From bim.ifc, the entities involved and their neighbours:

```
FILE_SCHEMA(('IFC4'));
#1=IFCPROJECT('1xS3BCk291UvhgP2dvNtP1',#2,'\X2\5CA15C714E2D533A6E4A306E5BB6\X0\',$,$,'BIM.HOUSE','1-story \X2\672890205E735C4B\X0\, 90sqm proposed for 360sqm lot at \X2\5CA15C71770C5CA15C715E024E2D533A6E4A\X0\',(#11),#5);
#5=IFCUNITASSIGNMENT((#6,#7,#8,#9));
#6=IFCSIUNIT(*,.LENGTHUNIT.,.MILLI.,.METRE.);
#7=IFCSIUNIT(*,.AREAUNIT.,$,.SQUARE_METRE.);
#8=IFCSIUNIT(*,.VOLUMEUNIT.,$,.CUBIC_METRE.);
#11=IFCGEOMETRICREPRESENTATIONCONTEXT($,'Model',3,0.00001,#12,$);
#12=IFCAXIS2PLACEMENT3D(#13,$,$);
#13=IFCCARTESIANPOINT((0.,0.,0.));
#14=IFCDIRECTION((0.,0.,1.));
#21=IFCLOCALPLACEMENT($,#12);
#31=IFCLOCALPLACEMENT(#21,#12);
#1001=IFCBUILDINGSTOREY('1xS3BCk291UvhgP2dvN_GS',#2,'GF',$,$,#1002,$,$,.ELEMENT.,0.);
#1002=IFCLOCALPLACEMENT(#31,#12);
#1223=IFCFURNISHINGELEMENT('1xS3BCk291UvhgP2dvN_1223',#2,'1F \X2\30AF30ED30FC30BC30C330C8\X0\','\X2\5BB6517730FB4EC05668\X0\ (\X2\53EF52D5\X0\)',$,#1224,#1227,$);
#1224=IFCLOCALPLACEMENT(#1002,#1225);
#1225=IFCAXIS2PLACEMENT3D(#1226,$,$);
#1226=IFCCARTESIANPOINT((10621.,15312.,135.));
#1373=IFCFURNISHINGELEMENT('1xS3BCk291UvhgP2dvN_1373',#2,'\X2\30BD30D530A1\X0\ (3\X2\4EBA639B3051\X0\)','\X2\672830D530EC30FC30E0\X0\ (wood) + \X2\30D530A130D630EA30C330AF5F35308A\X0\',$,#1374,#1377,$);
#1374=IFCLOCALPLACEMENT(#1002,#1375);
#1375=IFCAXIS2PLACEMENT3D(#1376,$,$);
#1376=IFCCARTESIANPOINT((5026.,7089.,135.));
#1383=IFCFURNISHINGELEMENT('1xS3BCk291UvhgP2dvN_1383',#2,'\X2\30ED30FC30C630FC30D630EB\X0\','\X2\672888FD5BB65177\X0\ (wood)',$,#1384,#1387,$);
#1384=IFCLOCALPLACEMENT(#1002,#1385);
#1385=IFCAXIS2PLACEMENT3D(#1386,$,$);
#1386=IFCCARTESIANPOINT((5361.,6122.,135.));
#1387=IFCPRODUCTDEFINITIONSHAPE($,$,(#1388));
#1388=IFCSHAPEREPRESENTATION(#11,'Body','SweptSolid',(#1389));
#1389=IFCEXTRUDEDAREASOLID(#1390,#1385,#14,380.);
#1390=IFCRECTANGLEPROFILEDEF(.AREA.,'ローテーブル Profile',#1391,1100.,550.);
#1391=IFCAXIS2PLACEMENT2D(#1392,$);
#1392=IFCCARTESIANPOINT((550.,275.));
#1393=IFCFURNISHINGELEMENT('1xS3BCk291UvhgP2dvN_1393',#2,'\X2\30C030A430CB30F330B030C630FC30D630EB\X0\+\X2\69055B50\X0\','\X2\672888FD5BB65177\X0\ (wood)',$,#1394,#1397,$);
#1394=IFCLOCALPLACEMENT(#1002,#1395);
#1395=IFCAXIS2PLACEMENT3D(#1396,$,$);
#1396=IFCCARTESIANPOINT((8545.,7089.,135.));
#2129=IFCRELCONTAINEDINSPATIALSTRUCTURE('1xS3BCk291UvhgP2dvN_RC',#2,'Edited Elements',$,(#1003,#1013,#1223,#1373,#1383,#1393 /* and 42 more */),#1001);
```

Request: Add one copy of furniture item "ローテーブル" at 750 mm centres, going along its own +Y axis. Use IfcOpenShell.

```python
import ifcopenshell
import ifcopenshell.api.geometry
import ifcopenshell.api.root
import ifcopenshell.util.element
import ifcopenshell.util.placement

model = ifcopenshell.open("bim.ifc")


def reuse_history(source, copy):
    """copy_class also copies each property set's owner history, people and application; keep the originals."""
    for rel in copy.IsDefinedBy:
        if rel.is_a("IfcRelDefinesByProperties") and (history := rel.RelatingPropertyDefinition.OwnerHistory):
            rel.RelatingPropertyDefinition.OwnerHistory = source.OwnerHistory
            ifcopenshell.util.element.remove_deep2(model, history)


source = model.by_guid("1xS3BCk291UvhgP2dvN_1383")
base = ifcopenshell.util.placement.get_local_placement(source.ObjectPlacement)
step = base[:3, 1] * 750.0

for i in range(1, 2):
    copy = ifcopenshell.api.root.copy_class(model, product=source)
    copy.Representation = ifcopenshell.util.element.copy_deep(
        model, source.Representation, exclude=["IfcGeometricRepresentationContext", "IfcRepresentationMap"]
    )
    reuse_history(source, copy)
    matrix = base.copy()
    matrix[:3, 3] += i * step
    print("added at", matrix[:3, 3].round(3) + 0.0)
    ifcopenshell.api.geometry.edit_object_placement(model, product=copy, matrix=matrix, is_si=False)

model.write("bim_edited.ifc")
```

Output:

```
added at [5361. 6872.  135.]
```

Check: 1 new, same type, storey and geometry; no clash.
